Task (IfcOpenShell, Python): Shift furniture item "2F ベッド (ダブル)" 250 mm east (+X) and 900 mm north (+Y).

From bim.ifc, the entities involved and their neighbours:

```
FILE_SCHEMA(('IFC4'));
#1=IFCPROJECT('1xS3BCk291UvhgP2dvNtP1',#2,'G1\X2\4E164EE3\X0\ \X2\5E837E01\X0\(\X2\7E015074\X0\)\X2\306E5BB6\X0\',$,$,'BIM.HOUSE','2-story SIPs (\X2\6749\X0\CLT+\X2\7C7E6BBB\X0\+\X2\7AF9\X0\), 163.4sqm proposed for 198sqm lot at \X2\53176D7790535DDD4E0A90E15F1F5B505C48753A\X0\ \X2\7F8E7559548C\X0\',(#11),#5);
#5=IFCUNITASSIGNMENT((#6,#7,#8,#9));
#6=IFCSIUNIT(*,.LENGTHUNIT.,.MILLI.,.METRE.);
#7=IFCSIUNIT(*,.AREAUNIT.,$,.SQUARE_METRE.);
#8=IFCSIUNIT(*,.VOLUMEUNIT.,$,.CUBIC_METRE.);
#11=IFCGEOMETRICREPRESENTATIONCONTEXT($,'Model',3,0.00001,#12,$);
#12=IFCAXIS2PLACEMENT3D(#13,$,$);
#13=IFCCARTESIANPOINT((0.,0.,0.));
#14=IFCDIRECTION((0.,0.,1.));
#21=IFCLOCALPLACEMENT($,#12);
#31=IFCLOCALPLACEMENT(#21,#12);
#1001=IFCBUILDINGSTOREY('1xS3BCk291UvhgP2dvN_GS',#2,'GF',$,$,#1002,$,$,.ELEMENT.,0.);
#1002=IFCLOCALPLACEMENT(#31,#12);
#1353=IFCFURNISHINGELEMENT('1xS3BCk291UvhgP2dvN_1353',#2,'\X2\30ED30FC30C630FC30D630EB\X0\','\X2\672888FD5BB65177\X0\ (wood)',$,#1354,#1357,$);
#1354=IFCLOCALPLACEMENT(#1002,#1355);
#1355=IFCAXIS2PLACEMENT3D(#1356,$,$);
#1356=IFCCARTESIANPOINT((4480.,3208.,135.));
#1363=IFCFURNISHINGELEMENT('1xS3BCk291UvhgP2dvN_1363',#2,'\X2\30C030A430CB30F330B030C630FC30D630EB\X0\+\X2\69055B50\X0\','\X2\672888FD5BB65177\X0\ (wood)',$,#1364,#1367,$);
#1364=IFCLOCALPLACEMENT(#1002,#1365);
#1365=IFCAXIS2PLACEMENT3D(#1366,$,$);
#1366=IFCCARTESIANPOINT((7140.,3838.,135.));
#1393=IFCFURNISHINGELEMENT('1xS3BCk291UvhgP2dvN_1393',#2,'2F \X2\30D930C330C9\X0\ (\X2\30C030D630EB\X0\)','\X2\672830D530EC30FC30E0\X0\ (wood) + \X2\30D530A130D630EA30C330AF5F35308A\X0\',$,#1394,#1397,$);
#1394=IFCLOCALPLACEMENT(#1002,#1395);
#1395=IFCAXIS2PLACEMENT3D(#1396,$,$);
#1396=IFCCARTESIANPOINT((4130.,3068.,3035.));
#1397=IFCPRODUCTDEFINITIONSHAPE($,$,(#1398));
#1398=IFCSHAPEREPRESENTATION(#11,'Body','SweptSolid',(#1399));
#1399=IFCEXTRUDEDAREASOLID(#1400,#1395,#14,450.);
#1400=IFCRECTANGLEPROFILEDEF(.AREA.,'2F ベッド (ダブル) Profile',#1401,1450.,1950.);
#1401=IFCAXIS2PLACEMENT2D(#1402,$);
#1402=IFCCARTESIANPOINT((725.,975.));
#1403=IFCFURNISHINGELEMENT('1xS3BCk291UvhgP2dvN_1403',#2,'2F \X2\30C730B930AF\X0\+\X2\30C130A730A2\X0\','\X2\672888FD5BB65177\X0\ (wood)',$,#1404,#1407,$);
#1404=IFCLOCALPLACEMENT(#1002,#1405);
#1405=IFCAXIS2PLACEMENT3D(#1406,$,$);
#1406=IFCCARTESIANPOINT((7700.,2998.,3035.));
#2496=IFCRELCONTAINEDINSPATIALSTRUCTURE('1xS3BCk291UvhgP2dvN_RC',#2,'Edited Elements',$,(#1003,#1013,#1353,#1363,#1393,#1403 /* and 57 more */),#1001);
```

```python
import ifcopenshell
import ifcopenshell.api.geometry
import ifcopenshell.util.placement
import ifcopenshell.util.unit

model = ifcopenshell.open("bim.ifc")
unit_scale = ifcopenshell.util.unit.calculate_unit_scale(model)

item = model.by_id(1393)
matrix = ifcopenshell.util.placement.get_local_placement(item.ObjectPlacement)
matrix[0, 3] += 0.25 / unit_scale
matrix[1, 3] += 0.9 / unit_scale
ifcopenshell.api.geometry.edit_object_placement(model, product=item, matrix=matrix, is_si=False)

print(ifcopenshell.util.placement.get_local_placement(item.ObjectPlacement).round(3) + 0.0)

model.write("bim_v2.ifc")
```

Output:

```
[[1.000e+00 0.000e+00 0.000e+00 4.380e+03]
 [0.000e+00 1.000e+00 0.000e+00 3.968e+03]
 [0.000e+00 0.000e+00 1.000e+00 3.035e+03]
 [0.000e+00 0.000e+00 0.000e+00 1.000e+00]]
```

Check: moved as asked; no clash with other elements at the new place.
